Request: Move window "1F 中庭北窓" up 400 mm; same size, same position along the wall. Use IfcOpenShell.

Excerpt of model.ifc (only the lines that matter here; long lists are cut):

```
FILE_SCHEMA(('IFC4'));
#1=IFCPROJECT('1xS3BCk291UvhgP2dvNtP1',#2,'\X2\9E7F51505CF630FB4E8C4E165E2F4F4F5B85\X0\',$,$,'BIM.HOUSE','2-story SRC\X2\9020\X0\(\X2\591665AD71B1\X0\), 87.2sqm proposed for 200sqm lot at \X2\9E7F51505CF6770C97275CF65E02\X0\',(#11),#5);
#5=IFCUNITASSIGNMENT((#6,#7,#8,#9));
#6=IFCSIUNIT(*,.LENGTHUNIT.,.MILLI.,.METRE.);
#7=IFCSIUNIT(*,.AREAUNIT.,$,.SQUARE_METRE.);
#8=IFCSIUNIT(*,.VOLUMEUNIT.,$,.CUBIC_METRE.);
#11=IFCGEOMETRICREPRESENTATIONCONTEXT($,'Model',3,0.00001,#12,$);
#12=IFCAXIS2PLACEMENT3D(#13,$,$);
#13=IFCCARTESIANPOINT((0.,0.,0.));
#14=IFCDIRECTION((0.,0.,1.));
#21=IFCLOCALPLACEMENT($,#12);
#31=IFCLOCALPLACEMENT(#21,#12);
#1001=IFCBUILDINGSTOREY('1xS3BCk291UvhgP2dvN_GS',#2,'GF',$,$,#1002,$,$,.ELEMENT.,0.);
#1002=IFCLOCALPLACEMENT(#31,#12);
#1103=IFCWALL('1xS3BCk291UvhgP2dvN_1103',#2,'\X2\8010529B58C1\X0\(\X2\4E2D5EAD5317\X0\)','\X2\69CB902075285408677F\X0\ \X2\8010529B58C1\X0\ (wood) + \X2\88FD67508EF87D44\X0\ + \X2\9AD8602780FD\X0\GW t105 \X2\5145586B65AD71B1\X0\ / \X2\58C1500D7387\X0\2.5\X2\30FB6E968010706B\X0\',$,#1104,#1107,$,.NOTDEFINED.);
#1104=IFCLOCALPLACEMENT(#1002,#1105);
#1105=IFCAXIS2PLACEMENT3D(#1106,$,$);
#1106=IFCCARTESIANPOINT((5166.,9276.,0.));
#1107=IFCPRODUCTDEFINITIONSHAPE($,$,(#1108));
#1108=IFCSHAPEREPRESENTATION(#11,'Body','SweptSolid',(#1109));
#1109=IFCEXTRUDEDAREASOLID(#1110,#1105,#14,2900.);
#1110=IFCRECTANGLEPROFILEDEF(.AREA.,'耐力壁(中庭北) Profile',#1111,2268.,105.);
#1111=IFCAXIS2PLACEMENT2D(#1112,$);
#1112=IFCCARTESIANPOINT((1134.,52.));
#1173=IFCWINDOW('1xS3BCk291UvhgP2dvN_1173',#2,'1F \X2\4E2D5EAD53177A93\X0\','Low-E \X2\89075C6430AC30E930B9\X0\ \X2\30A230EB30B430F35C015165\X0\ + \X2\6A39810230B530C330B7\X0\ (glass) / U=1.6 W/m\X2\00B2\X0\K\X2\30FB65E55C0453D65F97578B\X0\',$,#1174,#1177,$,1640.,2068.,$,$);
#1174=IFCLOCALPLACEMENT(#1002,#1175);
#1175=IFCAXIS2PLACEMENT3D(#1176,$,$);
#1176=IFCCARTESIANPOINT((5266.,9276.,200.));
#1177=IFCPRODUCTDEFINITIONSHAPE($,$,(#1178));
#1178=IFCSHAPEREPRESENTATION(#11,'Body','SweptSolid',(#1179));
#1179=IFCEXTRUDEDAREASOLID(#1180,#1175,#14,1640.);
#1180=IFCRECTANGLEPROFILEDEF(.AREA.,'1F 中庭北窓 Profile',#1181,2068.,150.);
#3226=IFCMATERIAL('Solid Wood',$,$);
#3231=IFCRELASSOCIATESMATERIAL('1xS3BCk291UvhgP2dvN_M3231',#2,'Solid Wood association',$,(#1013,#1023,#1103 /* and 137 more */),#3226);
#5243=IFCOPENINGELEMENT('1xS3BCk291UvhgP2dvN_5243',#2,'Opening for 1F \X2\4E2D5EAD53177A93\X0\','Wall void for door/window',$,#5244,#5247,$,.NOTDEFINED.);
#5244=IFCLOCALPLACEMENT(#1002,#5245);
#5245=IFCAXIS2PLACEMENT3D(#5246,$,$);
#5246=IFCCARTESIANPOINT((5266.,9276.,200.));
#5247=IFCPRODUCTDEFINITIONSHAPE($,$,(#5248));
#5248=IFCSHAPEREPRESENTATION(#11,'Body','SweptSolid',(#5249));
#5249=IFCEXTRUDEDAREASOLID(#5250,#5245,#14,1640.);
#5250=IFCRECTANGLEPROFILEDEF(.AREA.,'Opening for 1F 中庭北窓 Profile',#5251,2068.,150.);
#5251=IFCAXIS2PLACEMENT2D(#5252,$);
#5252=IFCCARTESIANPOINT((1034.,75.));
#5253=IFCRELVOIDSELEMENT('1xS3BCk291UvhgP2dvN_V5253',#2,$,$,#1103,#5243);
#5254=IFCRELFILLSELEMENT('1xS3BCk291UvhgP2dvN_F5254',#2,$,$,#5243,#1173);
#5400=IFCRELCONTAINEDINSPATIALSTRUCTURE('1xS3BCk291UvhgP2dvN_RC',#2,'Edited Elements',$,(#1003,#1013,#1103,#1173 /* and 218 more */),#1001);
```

```python
import numpy as np
import ifcopenshell
import ifcopenshell.api.geometry
import ifcopenshell.util.placement
import ifcopenshell.util.unit

model = ifcopenshell.open("model.ifc")
unit_scale = ifcopenshell.util.unit.calculate_unit_scale(model)

window = model.by_guid("1xS3BCk291UvhgP2dvN_1173")
opening = window.FillsVoids[0].RelatingOpeningElement
dz = 400.0

shift = np.array([0.0, 0.0, dz])
# The window is not placed relative to its opening, so move both.
for product in (opening, window):
    matrix = ifcopenshell.util.placement.get_local_placement(product.ObjectPlacement)
    matrix[:3, 3] += shift
    ifcopenshell.api.geometry.edit_object_placement(model, product=product, matrix=matrix, is_si=False)

print(f"moved by {dz * unit_scale:+.3f} m")

model.write("model_edited.ifc")
```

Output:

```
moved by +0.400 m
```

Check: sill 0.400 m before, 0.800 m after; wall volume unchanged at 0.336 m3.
